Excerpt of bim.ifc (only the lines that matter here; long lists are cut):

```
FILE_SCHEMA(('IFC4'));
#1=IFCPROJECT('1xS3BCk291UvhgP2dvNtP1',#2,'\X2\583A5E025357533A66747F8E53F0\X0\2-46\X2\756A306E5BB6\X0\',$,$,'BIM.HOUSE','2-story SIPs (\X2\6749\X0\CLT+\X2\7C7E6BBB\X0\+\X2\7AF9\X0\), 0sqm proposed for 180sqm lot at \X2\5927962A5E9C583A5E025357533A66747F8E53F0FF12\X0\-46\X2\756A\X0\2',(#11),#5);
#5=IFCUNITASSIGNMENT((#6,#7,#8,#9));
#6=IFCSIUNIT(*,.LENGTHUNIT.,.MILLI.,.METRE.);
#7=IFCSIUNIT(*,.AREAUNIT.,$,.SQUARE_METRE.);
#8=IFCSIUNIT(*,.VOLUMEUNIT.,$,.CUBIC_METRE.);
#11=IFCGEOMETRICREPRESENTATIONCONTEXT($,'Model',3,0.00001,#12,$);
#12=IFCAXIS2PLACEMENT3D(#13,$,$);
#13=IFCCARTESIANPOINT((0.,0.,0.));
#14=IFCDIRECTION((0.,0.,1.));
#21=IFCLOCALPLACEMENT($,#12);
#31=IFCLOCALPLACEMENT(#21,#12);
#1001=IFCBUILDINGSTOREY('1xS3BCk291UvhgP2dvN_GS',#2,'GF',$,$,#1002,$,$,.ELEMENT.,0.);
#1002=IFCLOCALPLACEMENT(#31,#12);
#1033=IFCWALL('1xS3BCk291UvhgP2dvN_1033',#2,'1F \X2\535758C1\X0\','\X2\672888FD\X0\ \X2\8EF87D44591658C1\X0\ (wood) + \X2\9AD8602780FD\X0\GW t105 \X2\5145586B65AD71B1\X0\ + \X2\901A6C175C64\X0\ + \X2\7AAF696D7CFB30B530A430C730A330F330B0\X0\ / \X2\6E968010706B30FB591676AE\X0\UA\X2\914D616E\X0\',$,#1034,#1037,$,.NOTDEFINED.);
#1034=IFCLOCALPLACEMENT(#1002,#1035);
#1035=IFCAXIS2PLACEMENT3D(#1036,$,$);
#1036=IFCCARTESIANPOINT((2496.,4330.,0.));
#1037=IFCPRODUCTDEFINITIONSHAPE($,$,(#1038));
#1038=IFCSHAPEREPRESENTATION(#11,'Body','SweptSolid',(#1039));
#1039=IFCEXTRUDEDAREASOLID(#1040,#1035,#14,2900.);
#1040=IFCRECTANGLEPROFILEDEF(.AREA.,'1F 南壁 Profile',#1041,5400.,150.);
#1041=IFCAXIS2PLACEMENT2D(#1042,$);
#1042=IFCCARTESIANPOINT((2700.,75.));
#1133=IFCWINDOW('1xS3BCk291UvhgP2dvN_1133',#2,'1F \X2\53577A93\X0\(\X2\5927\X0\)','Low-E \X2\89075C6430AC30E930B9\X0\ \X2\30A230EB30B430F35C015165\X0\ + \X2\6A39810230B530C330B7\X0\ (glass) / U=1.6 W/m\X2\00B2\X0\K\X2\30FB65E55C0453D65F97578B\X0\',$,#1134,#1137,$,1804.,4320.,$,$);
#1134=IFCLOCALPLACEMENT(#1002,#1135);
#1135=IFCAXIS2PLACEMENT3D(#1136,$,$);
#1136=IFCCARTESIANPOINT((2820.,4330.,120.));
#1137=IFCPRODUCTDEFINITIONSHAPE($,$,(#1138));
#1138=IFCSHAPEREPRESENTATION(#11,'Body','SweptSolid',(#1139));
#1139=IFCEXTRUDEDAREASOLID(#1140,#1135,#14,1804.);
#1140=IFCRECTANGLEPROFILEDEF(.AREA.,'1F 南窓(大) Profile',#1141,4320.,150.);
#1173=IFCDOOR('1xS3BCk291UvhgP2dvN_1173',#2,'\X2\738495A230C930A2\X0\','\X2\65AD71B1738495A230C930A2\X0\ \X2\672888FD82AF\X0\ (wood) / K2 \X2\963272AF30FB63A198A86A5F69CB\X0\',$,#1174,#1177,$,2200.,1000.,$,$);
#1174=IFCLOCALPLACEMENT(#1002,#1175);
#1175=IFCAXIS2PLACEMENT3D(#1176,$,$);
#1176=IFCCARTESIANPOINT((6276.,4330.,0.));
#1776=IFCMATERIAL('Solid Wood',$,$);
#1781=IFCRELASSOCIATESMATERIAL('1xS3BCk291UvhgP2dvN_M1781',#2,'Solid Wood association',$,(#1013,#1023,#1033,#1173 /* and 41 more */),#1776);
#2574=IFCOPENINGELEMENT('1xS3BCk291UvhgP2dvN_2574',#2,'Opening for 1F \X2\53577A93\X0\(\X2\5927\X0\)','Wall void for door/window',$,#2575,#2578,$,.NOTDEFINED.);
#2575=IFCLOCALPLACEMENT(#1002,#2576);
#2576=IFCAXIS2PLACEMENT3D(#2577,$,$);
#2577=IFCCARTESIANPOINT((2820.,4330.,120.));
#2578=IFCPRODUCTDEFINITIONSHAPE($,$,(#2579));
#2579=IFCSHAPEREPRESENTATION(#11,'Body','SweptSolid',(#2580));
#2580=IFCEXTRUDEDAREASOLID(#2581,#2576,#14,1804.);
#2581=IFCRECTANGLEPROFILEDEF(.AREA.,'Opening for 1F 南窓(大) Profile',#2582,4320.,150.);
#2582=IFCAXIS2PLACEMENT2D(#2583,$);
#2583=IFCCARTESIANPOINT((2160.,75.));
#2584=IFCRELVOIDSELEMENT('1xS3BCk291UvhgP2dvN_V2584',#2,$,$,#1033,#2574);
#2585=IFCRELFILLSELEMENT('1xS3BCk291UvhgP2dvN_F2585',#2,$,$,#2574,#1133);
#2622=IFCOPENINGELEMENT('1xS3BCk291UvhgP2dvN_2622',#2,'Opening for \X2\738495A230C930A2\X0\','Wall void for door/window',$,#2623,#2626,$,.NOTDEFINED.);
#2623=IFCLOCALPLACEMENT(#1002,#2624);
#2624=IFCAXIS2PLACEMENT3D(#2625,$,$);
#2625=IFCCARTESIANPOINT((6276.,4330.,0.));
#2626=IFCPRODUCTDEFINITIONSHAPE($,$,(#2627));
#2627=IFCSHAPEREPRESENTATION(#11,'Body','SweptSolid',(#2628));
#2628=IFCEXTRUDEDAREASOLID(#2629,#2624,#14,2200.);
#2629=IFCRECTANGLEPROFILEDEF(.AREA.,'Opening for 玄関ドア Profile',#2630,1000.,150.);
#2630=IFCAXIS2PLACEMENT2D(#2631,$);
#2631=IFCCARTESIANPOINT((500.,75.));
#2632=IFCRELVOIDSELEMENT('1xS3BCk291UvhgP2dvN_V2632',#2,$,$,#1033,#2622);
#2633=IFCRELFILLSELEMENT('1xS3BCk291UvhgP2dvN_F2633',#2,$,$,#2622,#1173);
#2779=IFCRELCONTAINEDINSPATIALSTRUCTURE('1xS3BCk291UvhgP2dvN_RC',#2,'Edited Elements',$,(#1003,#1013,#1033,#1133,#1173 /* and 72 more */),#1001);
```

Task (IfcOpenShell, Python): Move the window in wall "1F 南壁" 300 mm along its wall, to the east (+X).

```python
import ifcopenshell
import ifcopenshell.api.geometry
import ifcopenshell.util.placement
import ifcopenshell.util.unit

model = ifcopenshell.open("bim.ifc")
unit_scale = ifcopenshell.util.unit.calculate_unit_scale(model)

window = model.by_guid("1xS3BCk291UvhgP2dvN_1133")
opening = window.FillsVoids[0].RelatingOpeningElement
wall = opening.VoidsElements[0].RelatingBuildingElement

wall_matrix = ifcopenshell.util.placement.get_local_placement(wall.ObjectPlacement)
shift = wall_matrix[:3, 0] * 0.3 / unit_scale
before = ifcopenshell.util.placement.get_local_placement(window.ObjectPlacement)[:3, 3].copy()

# The window is not placed relative to its opening, so move both.
for product in (opening, window):
    matrix = ifcopenshell.util.placement.get_local_placement(product.ObjectPlacement)
    matrix[:3, 3] += shift
    ifcopenshell.api.geometry.edit_object_placement(model, product=product, matrix=matrix, is_si=False)

after = ifcopenshell.util.placement.get_local_placement(window.ObjectPlacement)[:3, 3]
print("window moved by", (after - before).round(3) + 0.0)

model.write("bim_rev.ifc")
```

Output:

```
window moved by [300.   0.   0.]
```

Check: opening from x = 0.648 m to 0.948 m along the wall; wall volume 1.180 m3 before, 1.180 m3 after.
